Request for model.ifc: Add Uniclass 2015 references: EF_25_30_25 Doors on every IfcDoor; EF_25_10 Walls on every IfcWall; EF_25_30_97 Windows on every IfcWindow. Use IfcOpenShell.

First a look at what the model holds.

```python
import ifcopenshell

model = ifcopenshell.open("model.ifc")
print(model.schema)
print("classifications:", [c.Name for c in model.by_type("IfcClassification")])
for ifc_class in ("IfcDoor", "IfcRoof", "IfcStair", "IfcWall", "IfcWindow"):
    print(ifc_class, len(model.by_type(ifc_class)))
```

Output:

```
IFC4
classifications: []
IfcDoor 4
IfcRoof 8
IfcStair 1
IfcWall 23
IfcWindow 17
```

```python
import ifcopenshell
import ifcopenshell.api.classification

model = ifcopenshell.open("model.ifc")

system = ifcopenshell.api.classification.add_classification(model, classification="Uniclass 2015")

codes = {
    "IfcDoor": ("EF_25_30_25", "Doors"),
    "IfcWall": ("EF_25_10", "Walls"),
    "IfcWindow": ("EF_25_30_97", "Windows"),
}
for ifc_class, (code, name) in codes.items():
    products = model.by_type(ifc_class)
    ifcopenshell.api.classification.add_reference(
        model, products=products, classification=system, identification=code, name=name
    )
    print(code, len(products))

model.write("model-out.ifc")
```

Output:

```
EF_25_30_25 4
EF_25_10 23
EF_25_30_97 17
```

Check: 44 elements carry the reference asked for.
